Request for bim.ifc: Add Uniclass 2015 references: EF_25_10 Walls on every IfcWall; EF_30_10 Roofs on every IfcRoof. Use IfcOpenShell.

First a look at what the model holds.

```python
import ifcopenshell

model = ifcopenshell.open("bim.ifc")
print(model.schema)
print("classifications:", [c.Name for c in model.by_type("IfcClassification")])
for ifc_class in ("IfcDoor", "IfcRoof", "IfcStair", "IfcWall", "IfcWindow"):
    print(ifc_class, len(model.by_type(ifc_class)))
```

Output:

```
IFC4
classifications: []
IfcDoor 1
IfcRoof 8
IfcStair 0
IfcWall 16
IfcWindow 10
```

```python
import ifcopenshell
import ifcopenshell.api.classification

model = ifcopenshell.open("bim.ifc")

system = ifcopenshell.api.classification.add_classification(model, classification="Uniclass 2015")

codes = {
    "IfcWall": ("EF_25_10", "Walls"),
    "IfcRoof": ("EF_30_10", "Roofs"),
}
for ifc_class, (code, name) in codes.items():
    products = model.by_type(ifc_class)
    ifcopenshell.api.classification.add_reference(
        model, products=products, classification=system, identification=code, name=name
    )
    print(code, len(products))

model.write("bim_rev.ifc")
```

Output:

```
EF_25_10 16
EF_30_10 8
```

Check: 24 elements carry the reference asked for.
